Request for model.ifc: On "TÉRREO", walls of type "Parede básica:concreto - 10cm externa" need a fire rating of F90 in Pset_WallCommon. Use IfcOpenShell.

First a look at what the model holds.

```python
import ifcopenshell
import ifcopenshell.util.element

model = ifcopenshell.open("model.ifc")
print(model.schema)
storey = next(s for s in model.by_type("IfcBuildingStorey") if s.Name == "TÉRREO")
walls = [e for e in ifcopenshell.util.element.get_decomposition(storey) if e.is_a("IfcWall")]
seen = {}
for e in walls:
    element_type = ifcopenshell.util.element.get_type(e)
    key = (element_type.Name if element_type != e and element_type else None, ifcopenshell.util.element.get_pset(e, "Pset_WallCommon", "FireRating"))
    seen[key] = seen.get(key, 0) + 1
for (name, value), count in sorted(seen.items(), key=str):
    print(count, "x", name, "|", value)
```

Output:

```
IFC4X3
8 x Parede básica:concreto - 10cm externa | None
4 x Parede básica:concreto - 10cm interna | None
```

```python
import ifcopenshell
import ifcopenshell.api.pset
import ifcopenshell.util.element

model = ifcopenshell.open("model.ifc")

storey = next(s for s in model.by_type("IfcBuildingStorey") if s.Name == "TÉRREO")
walls = [e for e in ifcopenshell.util.element.get_decomposition(storey) if e.is_a("IfcWall")]

count = 0
for e in walls:
    element_type = ifcopenshell.util.element.get_type(e)
    if element_type in (None, e) or element_type.Name != "Parede básica:concreto - 10cm externa":
        continue
    # add_pset returns the element's existing set when there is one.
    pset = ifcopenshell.api.pset.add_pset(model, product=e, name="Pset_WallCommon")
    ifcopenshell.api.pset.edit_pset(model, pset=pset, properties={"FireRating": "F90"})
    count += 1

print(count, "walls updated")

model.write("model_v2.ifc")
```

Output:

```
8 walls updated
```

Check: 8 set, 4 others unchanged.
